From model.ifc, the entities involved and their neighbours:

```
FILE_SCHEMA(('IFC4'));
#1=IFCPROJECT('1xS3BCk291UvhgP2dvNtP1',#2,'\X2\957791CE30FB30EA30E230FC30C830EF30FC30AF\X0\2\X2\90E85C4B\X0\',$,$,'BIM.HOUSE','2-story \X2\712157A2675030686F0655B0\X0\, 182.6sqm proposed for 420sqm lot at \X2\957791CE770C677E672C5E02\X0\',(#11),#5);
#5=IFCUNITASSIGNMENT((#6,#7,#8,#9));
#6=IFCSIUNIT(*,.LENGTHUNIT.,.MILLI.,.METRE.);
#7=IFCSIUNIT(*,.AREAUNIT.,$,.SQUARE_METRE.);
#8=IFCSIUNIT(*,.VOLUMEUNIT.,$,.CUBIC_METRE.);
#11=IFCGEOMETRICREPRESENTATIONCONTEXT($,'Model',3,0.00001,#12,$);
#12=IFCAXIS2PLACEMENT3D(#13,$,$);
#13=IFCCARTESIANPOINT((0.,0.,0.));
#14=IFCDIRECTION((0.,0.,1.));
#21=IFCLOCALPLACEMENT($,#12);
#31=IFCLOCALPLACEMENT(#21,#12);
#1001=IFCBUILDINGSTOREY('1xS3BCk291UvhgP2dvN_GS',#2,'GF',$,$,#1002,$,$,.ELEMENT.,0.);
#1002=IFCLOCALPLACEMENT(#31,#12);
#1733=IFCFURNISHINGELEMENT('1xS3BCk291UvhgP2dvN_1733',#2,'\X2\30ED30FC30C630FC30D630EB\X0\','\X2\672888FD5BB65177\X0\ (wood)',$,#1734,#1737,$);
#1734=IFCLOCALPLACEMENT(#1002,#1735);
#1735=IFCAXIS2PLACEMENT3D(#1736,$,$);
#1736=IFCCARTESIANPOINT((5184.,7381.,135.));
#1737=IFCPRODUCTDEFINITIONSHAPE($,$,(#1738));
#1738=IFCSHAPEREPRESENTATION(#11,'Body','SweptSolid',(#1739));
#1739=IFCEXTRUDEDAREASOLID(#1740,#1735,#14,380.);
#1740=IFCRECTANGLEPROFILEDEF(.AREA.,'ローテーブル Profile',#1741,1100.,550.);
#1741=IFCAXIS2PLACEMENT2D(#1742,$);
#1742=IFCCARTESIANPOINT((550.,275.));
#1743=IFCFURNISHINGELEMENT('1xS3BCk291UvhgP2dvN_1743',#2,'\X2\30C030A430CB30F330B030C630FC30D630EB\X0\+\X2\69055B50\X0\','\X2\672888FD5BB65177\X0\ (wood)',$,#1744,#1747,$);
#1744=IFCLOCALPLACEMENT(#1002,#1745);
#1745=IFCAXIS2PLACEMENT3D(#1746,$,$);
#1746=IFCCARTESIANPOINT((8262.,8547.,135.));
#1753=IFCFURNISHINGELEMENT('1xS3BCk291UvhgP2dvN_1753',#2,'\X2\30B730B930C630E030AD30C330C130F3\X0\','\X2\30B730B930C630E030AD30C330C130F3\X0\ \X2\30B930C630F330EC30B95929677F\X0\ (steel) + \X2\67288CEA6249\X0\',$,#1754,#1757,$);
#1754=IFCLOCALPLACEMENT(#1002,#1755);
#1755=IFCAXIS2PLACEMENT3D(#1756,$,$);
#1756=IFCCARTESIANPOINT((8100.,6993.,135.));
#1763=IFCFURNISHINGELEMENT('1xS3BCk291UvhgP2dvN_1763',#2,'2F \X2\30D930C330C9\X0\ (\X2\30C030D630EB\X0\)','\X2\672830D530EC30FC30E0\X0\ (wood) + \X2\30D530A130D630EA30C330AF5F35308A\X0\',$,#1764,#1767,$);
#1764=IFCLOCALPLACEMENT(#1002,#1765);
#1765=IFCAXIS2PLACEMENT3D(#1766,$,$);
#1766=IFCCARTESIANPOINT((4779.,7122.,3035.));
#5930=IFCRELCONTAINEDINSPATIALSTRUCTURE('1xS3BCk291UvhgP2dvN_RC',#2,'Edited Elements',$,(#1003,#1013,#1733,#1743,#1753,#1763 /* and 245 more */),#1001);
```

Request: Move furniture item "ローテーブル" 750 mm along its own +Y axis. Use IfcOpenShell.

```python
import ifcopenshell
import ifcopenshell.api.geometry
import ifcopenshell.util.placement
import ifcopenshell.util.unit

model = ifcopenshell.open("model.ifc")
unit_scale = ifcopenshell.util.unit.calculate_unit_scale(model)

item = model.by_guid("1xS3BCk291UvhgP2dvN_1733")
matrix = ifcopenshell.util.placement.get_local_placement(item.ObjectPlacement)
matrix[:3, 3] += matrix[:3, 1] * 0.75 / unit_scale
ifcopenshell.api.geometry.edit_object_placement(model, product=item, matrix=matrix, is_si=False)

print(ifcopenshell.util.placement.get_local_placement(item.ObjectPlacement).round(3) + 0.0)

model.write("model_updated.ifc")
```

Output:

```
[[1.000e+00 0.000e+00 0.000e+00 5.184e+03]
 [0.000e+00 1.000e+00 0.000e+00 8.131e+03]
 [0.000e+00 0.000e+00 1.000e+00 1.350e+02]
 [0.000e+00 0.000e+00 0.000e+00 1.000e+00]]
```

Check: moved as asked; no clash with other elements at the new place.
